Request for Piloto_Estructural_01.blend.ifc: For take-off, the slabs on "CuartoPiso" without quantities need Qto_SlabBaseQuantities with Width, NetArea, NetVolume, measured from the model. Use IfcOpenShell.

First a look at what the model holds.

```python
import ifcopenshell
import ifcopenshell.util.element
import ifcopenshell.util.unit

model = ifcopenshell.open("Piloto_Estructural_01.blend.ifc")
print(model.schema)
for unit_type in ("LENGTHUNIT", "AREAUNIT", "VOLUMEUNIT"):
    print(unit_type, ifcopenshell.util.unit.calculate_unit_scale(model, unit_type))
storey = next(s for s in model.by_type("IfcBuildingStorey") if s.Name == "CuartoPiso")
slabs = [e for e in ifcopenshell.util.element.get_decomposition(storey) if e.is_a("IfcSlab")]
for e in sorted(slabs, key=lambda e: e.id()):
    print(e.id(), e.is_a(), e.Name, list(ifcopenshell.util.element.get_psets(e, qtos_only=True)), sep=" | ")
```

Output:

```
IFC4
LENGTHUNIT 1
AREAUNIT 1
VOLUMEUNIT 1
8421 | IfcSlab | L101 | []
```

```python
import ifcopenshell
import ifcopenshell.api.pset
import ifcopenshell.geom
import ifcopenshell.util.element
import ifcopenshell.util.shape
import ifcopenshell.util.unit

model = ifcopenshell.open("Piloto_Estructural_01.blend.ifc")
unit_scale = ifcopenshell.util.unit.calculate_unit_scale(model)
area_scale = ifcopenshell.util.unit.calculate_unit_scale(model, "AREAUNIT")
volume_scale = ifcopenshell.util.unit.calculate_unit_scale(model, "VOLUMEUNIT")
settings = ifcopenshell.geom.settings()

storey = next(s for s in model.by_type("IfcBuildingStorey") if s.Name == "CuartoPiso")
slabs = [e for e in ifcopenshell.util.element.get_decomposition(storey) if e.is_a("IfcSlab")]

for e in sorted(slabs, key=lambda e: e.id()):
    if ifcopenshell.util.element.get_psets(e, qtos_only=True, should_inherit=False):
        continue
    # Geometry comes back in metres, in the element's own axes.
    shape = ifcopenshell.geom.create_shape(settings, e)
    values = {
        "Width": ifcopenshell.util.shape.get_z(shape.geometry) / unit_scale,
        "NetArea": ifcopenshell.util.shape.get_footprint_area(shape.geometry) / area_scale,
        "NetVolume": ifcopenshell.util.shape.get_volume(shape.geometry) / volume_scale,
    }
    qto = ifcopenshell.api.pset.add_qto(model, product=e, name="Qto_SlabBaseQuantities")
    ifcopenshell.api.pset.edit_qto(model, qto=qto, properties=values)
    print(e.id(), {k: round(v, 3) for k, v in values.items()})

model.write("Piloto_Estructural_01.blend_updated.ifc")
```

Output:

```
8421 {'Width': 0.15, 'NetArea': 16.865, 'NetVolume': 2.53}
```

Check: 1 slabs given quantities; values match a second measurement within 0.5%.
